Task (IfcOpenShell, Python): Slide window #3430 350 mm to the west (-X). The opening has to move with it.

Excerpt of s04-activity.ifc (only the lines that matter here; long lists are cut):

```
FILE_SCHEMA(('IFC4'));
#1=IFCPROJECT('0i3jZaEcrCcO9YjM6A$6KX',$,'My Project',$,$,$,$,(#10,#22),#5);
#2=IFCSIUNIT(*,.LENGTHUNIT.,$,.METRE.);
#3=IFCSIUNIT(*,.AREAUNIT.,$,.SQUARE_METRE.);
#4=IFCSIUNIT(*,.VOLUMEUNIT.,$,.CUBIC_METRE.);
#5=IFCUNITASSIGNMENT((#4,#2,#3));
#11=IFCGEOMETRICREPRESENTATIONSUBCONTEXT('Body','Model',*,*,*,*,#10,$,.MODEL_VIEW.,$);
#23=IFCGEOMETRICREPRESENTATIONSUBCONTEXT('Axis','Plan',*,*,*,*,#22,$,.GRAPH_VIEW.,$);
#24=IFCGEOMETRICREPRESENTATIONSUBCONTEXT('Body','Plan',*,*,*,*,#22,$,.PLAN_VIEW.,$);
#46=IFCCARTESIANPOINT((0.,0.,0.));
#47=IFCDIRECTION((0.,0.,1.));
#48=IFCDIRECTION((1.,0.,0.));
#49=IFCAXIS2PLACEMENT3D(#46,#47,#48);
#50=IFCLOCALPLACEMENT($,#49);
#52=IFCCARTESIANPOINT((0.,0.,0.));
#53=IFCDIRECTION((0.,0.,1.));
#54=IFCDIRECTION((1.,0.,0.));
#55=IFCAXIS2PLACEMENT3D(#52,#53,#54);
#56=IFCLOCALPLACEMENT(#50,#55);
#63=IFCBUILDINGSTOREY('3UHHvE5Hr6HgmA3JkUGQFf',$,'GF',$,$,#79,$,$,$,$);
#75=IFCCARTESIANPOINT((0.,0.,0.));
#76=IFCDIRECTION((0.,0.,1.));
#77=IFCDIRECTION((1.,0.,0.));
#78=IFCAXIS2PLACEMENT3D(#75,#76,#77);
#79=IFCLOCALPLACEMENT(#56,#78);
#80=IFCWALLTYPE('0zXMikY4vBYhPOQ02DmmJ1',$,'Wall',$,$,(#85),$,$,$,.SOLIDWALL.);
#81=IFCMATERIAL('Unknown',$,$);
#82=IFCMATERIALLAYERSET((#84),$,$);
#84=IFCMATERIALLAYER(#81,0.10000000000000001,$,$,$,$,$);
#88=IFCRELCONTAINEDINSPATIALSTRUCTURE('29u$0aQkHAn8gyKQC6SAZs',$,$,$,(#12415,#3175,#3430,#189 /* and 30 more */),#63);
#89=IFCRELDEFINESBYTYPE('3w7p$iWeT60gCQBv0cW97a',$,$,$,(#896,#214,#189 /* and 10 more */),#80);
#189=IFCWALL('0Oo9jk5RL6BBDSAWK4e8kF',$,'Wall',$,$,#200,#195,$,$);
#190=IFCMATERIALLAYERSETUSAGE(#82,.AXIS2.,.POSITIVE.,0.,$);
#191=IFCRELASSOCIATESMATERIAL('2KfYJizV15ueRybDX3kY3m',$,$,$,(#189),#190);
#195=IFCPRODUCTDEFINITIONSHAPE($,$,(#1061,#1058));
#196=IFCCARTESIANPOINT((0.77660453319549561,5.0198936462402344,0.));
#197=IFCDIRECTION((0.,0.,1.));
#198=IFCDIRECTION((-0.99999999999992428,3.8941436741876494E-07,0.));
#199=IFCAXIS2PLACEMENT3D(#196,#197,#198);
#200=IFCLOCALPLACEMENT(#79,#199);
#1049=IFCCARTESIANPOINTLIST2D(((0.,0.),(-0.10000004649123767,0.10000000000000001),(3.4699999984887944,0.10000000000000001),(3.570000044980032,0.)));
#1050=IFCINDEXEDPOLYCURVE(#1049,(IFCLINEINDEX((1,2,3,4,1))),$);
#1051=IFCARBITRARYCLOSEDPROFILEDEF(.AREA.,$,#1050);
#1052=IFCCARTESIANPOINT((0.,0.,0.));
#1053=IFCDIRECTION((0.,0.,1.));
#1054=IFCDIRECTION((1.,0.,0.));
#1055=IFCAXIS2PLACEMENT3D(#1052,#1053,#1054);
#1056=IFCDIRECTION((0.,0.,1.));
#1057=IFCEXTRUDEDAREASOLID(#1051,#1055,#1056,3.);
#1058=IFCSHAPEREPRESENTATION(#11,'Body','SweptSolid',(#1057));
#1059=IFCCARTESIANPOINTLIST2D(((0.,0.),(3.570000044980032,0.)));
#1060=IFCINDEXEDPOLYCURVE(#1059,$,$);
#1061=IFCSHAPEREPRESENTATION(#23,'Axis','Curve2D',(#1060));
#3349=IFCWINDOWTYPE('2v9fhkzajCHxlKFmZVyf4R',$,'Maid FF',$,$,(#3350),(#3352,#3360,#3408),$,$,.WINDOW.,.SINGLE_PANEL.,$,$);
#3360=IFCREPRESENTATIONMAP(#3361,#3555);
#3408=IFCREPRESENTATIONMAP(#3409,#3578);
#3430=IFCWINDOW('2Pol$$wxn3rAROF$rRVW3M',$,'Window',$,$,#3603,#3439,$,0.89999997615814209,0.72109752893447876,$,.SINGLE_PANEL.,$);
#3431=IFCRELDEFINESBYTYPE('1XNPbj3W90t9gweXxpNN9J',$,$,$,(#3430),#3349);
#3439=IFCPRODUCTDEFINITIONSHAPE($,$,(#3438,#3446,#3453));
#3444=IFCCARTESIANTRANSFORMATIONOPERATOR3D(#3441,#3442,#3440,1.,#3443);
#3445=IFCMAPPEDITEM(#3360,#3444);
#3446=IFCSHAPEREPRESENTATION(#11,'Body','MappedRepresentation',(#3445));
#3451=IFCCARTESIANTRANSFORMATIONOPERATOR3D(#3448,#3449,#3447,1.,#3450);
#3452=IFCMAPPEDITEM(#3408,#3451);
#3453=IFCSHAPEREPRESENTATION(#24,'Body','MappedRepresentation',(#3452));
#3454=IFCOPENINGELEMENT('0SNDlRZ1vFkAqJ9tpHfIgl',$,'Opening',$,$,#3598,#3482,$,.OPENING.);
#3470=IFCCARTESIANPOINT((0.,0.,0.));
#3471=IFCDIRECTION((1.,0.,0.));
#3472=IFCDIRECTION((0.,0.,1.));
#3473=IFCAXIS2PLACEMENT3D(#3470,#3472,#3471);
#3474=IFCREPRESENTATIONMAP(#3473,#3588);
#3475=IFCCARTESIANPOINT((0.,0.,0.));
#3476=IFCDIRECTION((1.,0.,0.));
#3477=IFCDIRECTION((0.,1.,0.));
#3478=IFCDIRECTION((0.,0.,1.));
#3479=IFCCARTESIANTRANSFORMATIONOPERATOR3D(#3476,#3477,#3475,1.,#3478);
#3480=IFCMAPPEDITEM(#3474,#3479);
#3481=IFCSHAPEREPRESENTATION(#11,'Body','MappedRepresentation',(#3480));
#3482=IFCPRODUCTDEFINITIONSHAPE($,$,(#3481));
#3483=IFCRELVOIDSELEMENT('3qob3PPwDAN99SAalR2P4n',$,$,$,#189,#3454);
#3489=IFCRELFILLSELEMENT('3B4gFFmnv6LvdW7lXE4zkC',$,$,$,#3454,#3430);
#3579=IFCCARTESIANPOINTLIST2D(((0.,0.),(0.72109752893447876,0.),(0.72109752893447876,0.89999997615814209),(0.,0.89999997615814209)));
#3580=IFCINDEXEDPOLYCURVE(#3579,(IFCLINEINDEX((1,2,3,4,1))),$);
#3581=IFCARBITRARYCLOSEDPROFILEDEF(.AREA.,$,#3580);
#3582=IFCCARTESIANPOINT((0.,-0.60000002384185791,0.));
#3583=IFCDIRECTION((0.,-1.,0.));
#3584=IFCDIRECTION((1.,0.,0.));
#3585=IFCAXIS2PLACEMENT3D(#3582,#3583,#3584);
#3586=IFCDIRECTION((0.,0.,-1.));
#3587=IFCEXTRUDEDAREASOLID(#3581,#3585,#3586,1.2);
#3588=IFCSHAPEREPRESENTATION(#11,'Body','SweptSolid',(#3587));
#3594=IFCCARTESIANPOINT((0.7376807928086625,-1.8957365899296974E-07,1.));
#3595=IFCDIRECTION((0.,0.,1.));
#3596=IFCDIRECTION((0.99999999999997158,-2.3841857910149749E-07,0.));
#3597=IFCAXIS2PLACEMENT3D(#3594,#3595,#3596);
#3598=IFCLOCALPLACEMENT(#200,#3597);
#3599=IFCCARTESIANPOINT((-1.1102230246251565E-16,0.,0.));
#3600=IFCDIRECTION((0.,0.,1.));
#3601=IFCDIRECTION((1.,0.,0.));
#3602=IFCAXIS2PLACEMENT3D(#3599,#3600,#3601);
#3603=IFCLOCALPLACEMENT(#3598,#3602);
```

```python
import ifcopenshell
import ifcopenshell.api.geometry
import ifcopenshell.util.placement
import ifcopenshell.util.unit

model = ifcopenshell.open("s04-activity.ifc")
unit_scale = ifcopenshell.util.unit.calculate_unit_scale(model)

window = model.by_id(3430)
opening = window.FillsVoids[0].RelatingOpeningElement
wall = opening.VoidsElements[0].RelatingBuildingElement

wall_matrix = ifcopenshell.util.placement.get_local_placement(wall.ObjectPlacement)
shift = wall_matrix[:3, 0] * 0.35 / unit_scale
before = ifcopenshell.util.placement.get_local_placement(window.ObjectPlacement)[:3, 3].copy()

# The window is placed relative to its opening, so it follows when the opening moves.
matrix = ifcopenshell.util.placement.get_local_placement(opening.ObjectPlacement)
matrix[:3, 3] += shift
ifcopenshell.api.geometry.edit_object_placement(
    model, product=opening, matrix=matrix, is_si=False, should_transform_children=True
)

after = ifcopenshell.util.placement.get_local_placement(window.ObjectPlacement)[:3, 3]
print("window moved by", (after - before).round(3) + 0.0)

model.write("s04-activity-out.ifc")
```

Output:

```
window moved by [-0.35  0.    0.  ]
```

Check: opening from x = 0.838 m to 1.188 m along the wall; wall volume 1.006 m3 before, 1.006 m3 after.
